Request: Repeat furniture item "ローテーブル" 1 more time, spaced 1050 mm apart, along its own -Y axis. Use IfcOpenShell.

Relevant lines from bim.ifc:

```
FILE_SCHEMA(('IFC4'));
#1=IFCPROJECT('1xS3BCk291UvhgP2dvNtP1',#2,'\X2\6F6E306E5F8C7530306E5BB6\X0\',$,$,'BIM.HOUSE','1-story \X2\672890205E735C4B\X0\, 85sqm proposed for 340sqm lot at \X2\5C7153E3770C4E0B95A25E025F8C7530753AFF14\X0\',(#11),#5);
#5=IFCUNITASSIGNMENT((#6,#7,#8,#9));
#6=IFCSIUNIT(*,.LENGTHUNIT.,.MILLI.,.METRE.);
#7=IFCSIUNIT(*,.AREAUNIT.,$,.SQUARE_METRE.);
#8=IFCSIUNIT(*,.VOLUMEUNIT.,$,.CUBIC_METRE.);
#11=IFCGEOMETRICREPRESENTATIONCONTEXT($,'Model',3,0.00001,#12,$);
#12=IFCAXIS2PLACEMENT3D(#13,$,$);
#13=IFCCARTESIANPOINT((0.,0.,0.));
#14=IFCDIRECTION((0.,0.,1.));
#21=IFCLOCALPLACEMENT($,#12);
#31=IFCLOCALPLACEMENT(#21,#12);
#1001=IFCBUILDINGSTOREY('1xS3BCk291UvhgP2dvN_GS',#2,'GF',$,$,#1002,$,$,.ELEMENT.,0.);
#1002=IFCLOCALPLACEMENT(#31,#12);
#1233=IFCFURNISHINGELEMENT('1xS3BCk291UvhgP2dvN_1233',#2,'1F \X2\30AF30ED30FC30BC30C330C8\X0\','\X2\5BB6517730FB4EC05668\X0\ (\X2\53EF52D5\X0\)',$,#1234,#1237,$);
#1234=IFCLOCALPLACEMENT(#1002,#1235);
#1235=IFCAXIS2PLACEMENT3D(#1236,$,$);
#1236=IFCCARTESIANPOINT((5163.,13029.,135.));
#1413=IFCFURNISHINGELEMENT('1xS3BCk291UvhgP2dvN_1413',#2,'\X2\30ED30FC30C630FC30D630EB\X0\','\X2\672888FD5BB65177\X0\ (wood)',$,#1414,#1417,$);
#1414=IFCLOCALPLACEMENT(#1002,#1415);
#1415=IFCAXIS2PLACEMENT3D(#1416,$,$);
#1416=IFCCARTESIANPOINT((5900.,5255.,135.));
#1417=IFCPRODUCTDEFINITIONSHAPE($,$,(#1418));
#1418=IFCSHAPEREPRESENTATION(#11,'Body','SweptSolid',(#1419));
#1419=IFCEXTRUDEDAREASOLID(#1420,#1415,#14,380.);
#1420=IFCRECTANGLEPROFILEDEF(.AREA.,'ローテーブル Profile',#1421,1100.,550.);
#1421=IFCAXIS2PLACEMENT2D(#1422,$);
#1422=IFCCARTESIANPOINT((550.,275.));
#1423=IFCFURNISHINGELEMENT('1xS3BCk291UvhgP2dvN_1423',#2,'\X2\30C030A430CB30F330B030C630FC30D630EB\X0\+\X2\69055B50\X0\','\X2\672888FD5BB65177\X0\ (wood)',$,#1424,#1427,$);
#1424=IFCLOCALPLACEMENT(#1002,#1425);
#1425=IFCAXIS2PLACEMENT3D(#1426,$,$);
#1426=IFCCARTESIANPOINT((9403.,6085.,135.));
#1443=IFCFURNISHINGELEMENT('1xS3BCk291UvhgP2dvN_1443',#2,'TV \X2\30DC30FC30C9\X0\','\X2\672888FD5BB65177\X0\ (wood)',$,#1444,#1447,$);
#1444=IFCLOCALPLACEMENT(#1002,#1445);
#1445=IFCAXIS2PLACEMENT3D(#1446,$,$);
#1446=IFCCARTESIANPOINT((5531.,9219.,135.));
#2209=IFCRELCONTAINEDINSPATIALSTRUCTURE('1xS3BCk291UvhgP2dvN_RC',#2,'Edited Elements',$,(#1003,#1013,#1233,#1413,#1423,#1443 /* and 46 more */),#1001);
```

```python
import ifcopenshell
import ifcopenshell.api.geometry
import ifcopenshell.api.root
import ifcopenshell.util.element
import ifcopenshell.util.placement
import ifcopenshell.util.unit

model = ifcopenshell.open("bim.ifc")
unit_scale = ifcopenshell.util.unit.calculate_unit_scale(model)


def reuse_history(source, copy):
    """copy_class also copies each property set's owner history, people and application; keep the originals."""
    for rel in copy.IsDefinedBy:
        if rel.is_a("IfcRelDefinesByProperties") and (history := rel.RelatingPropertyDefinition.OwnerHistory):
            rel.RelatingPropertyDefinition.OwnerHistory = source.OwnerHistory
            ifcopenshell.util.element.remove_deep2(model, history)


source = model.by_guid("1xS3BCk291UvhgP2dvN_1413")
base = ifcopenshell.util.placement.get_local_placement(source.ObjectPlacement)
step = -base[:3, 1] * 1.05 / unit_scale

for i in range(1, 2):
    copy = ifcopenshell.api.root.copy_class(model, product=source)
    copy.Representation = ifcopenshell.util.element.copy_deep(
        model, source.Representation, exclude=["IfcGeometricRepresentationContext", "IfcRepresentationMap"]
    )
    reuse_history(source, copy)
    matrix = base.copy()
    matrix[:3, 3] += i * step
    print("added at", matrix[:3, 3].round(3) + 0.0)
    ifcopenshell.api.geometry.edit_object_placement(model, product=copy, matrix=matrix, is_si=False)

model.write("bim_v2.ifc")
```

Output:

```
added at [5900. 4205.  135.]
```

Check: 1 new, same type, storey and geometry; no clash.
